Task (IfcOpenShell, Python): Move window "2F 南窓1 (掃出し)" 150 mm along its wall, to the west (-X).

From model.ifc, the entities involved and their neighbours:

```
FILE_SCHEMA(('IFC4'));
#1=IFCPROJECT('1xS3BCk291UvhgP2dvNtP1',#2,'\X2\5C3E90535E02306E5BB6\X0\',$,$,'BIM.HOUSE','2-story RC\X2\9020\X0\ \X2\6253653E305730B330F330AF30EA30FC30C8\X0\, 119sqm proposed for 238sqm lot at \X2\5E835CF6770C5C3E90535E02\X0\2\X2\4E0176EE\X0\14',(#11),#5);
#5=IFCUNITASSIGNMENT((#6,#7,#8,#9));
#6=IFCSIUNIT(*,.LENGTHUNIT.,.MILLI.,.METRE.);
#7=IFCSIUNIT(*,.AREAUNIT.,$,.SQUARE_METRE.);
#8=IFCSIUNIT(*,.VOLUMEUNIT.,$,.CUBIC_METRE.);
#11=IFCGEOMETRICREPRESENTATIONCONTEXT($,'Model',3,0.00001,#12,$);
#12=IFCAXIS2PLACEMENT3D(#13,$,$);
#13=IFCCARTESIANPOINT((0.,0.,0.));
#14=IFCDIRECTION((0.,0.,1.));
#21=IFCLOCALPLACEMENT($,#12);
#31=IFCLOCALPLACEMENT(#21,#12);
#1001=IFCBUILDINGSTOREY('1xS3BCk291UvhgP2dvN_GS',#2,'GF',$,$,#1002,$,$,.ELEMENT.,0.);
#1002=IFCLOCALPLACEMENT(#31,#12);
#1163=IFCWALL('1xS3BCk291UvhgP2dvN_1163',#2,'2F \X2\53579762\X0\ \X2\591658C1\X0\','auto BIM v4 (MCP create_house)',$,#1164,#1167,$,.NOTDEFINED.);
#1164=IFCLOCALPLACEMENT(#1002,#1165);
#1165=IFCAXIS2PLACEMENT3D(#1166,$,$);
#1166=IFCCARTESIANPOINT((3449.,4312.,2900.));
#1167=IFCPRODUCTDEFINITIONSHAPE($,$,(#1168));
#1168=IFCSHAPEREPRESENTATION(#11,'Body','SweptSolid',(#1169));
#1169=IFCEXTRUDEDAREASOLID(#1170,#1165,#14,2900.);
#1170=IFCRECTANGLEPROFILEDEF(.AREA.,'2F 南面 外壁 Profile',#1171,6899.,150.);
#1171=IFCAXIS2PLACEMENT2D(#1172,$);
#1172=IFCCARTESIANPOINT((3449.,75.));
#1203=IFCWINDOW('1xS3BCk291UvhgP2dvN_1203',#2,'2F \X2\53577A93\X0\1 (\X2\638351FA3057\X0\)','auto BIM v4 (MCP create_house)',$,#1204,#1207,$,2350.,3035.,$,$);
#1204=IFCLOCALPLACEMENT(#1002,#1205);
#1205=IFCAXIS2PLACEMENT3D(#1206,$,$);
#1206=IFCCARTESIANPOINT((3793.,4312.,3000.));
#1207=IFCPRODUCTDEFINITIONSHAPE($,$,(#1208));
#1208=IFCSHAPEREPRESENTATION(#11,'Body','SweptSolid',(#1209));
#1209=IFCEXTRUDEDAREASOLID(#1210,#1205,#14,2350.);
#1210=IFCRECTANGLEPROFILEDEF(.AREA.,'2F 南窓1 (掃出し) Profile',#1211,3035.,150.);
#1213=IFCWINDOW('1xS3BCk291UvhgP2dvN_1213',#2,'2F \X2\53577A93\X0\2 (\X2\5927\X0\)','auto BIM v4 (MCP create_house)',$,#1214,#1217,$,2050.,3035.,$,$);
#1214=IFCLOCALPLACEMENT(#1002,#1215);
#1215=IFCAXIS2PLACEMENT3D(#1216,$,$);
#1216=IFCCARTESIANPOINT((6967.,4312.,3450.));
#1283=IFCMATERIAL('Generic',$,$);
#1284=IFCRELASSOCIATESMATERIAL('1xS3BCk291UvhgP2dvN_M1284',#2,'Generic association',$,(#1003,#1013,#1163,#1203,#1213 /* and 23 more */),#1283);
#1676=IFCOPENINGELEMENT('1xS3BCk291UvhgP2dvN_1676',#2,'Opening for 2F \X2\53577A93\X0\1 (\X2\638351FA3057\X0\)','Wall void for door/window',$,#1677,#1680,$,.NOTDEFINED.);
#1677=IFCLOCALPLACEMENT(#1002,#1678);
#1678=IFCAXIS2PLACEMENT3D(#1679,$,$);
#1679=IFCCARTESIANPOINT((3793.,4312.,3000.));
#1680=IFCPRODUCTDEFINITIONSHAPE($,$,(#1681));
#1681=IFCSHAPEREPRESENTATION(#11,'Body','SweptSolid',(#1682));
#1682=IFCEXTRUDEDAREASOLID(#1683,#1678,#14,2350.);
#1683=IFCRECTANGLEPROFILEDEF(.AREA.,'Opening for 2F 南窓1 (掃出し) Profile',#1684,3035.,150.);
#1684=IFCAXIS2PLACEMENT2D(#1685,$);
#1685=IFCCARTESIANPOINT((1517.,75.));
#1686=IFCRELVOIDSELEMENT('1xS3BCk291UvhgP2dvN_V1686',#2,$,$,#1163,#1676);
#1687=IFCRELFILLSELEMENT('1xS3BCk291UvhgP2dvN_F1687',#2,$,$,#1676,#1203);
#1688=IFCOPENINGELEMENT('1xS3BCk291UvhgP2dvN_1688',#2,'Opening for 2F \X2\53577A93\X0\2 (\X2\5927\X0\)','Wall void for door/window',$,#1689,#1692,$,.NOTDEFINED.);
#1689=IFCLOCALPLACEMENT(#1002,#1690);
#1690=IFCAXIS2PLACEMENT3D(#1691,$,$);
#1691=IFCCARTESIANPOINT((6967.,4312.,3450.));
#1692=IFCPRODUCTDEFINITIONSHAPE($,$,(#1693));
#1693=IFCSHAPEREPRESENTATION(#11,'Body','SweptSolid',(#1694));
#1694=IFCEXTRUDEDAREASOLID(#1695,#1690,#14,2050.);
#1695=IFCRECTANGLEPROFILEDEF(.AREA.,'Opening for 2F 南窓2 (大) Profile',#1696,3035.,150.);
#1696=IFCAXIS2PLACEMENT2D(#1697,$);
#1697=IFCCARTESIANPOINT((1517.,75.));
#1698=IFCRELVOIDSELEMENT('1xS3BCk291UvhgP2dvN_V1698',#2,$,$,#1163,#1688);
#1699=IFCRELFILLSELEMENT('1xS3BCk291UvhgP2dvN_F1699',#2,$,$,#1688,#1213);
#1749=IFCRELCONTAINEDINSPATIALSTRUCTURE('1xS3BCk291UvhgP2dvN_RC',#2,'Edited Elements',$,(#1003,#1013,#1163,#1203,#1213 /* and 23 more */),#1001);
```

```python
import ifcopenshell
import ifcopenshell.api.geometry
import ifcopenshell.util.placement

model = ifcopenshell.open("model.ifc")

window = model.by_id(1203)
opening = window.FillsVoids[0].RelatingOpeningElement
wall = opening.VoidsElements[0].RelatingBuildingElement

wall_matrix = ifcopenshell.util.placement.get_local_placement(wall.ObjectPlacement)
shift = wall_matrix[:3, 0] * -150.0
before = ifcopenshell.util.placement.get_local_placement(window.ObjectPlacement)[:3, 3].copy()

# The window is not placed relative to its opening, so move both.
for product in (opening, window):
    matrix = ifcopenshell.util.placement.get_local_placement(product.ObjectPlacement)
    matrix[:3, 3] += shift
    ifcopenshell.api.geometry.edit_object_placement(model, product=product, matrix=matrix, is_si=False)

after = ifcopenshell.util.placement.get_local_placement(window.ObjectPlacement)[:3, 3]
print("window moved by", (after - before).round(3) + 0.0)

model.write("model_edited.ifc")
```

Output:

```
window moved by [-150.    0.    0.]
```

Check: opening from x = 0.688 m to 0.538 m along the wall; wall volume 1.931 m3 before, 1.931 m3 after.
